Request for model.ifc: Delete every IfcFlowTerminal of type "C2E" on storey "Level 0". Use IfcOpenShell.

First a look at what the model holds.

```python
import ifcopenshell
import ifcopenshell.util.element

model = ifcopenshell.open("model.ifc")
print(model.schema)
storey = next(s for s in model.by_type("IfcBuildingStorey") if s.Name == "Level 0")
terminals = [e for e in ifcopenshell.util.element.get_decomposition(storey) if e.is_a("IfcFlowTerminal")]
seen = {}
for e in terminals:
    element_type = ifcopenshell.util.element.get_type(e)
    name = element_type.Name if element_type not in (None, e) else None
    seen[name] = seen.get(name, 0) + 1
for name, count in sorted(seen.items(), key=str):
    print(count, "x", name)
```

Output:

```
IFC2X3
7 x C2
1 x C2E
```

```python
import ifcopenshell
import ifcopenshell.api.root
import ifcopenshell.util.element

model = ifcopenshell.open("model.ifc")

storey = next(s for s in model.by_type("IfcBuildingStorey") if s.Name == "Level 0")
terminals = [e for e in ifcopenshell.util.element.get_decomposition(storey) if e.is_a("IfcFlowTerminal")]
targets = [e for e in terminals if (t := ifcopenshell.util.element.get_type(e)) not in (None, e) and t.Name == "C2E"]

for e in targets:
    ifcopenshell.api.root.remove_product(model, product=e)
print(len(targets), "removed")

model.write("model_updated.ifc")
```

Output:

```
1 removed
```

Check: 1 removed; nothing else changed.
